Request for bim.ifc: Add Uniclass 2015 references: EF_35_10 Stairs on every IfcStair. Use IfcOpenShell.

First a look at what the model holds.

```python
import ifcopenshell

model = ifcopenshell.open("bim.ifc")
print(model.schema)
print("classifications:", [c.Name for c in model.by_type("IfcClassification")])
for ifc_class in ("IfcDoor", "IfcRoof", "IfcStair", "IfcWall", "IfcWindow"):
    print(ifc_class, len(model.by_type(ifc_class)))
```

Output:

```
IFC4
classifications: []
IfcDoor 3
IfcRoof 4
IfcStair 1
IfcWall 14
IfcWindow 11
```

```python
import ifcopenshell
import ifcopenshell.api.classification

model = ifcopenshell.open("bim.ifc")

system = ifcopenshell.api.classification.add_classification(model, classification="Uniclass 2015")

codes = {
    "IfcStair": ("EF_35_10", "Stairs"),
}
for ifc_class, (code, name) in codes.items():
    products = model.by_type(ifc_class)
    ifcopenshell.api.classification.add_reference(
        model, products=products, classification=system, identification=code, name=name
    )
    print(code, len(products))

model.write("bim_v2.ifc")
```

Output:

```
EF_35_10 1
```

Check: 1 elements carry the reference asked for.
